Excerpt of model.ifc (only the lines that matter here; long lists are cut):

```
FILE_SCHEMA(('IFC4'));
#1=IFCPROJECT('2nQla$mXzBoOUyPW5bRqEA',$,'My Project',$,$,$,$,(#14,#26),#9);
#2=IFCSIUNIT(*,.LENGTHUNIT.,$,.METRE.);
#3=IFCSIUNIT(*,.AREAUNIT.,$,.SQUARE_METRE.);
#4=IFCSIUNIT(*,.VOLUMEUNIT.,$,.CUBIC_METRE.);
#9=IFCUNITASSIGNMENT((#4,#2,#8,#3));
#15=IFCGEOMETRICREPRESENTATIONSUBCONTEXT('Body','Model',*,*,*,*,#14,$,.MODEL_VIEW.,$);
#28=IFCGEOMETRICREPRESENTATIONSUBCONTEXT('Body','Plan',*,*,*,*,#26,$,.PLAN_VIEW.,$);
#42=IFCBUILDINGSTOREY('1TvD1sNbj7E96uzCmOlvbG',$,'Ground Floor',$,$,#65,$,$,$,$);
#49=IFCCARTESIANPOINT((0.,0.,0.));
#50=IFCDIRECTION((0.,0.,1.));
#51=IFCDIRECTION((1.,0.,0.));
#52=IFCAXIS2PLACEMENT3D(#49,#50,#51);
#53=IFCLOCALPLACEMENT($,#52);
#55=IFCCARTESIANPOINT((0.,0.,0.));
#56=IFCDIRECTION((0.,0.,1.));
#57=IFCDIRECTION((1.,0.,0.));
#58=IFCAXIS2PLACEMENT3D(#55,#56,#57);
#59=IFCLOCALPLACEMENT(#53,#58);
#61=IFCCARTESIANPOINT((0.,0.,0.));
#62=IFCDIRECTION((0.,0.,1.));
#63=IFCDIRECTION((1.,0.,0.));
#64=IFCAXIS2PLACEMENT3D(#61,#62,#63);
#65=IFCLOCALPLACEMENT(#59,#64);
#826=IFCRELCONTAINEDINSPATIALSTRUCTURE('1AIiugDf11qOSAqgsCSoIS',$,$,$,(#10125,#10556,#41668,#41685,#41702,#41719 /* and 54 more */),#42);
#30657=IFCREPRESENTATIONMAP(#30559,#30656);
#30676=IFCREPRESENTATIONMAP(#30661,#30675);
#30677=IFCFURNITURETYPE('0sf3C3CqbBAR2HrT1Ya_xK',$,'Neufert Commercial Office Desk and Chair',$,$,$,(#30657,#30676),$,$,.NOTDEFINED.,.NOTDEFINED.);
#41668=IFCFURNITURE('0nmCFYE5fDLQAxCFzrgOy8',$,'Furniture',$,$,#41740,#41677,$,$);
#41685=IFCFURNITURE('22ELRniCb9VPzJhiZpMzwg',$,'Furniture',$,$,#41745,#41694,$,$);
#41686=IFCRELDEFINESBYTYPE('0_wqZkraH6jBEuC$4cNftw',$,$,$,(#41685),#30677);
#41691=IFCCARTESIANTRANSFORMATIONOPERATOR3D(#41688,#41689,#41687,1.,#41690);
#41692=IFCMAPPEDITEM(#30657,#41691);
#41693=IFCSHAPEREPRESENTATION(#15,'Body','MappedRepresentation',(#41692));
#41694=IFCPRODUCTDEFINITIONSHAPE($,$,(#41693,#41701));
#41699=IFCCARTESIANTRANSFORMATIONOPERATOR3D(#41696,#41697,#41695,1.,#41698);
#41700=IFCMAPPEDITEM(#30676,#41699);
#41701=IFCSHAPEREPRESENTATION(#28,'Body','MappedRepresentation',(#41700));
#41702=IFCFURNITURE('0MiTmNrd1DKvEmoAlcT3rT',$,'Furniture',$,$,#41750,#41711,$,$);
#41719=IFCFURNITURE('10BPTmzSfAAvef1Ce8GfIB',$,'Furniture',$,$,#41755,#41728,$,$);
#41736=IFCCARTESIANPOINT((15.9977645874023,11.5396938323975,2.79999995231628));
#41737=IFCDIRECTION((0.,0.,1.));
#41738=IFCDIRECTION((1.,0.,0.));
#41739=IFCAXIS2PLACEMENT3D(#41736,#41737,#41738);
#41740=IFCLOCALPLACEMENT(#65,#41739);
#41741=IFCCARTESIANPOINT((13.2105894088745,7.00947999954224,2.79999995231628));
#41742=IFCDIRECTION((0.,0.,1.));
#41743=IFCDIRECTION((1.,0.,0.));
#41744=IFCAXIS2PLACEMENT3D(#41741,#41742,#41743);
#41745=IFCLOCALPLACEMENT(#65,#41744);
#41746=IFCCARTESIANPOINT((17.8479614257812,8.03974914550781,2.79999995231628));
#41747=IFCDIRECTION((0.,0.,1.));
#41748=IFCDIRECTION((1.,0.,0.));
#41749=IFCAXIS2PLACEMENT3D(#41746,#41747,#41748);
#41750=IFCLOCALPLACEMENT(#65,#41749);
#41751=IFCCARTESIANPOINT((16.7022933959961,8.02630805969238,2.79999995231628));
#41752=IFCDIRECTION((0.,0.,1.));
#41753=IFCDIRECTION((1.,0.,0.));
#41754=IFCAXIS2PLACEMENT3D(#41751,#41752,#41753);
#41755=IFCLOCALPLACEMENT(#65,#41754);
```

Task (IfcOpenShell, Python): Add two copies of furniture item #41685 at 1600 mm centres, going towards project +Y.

```python
import numpy as np
import ifcopenshell
import ifcopenshell.api.geometry
import ifcopenshell.api.root
import ifcopenshell.util.element
import ifcopenshell.util.placement
import ifcopenshell.util.unit

model = ifcopenshell.open("model.ifc")
unit_scale = ifcopenshell.util.unit.calculate_unit_scale(model)

source = model.by_id(41685)
base = ifcopenshell.util.placement.get_local_placement(source.ObjectPlacement)
step = np.array([0.0, 1.0, 0.0]) * 1.6 / unit_scale

for i in range(1, 3):
    copy = ifcopenshell.api.root.copy_class(model, product=source)
    copy.Representation = ifcopenshell.util.element.copy_deep(
        model, source.Representation, exclude=["IfcGeometricRepresentationContext", "IfcRepresentationMap"]
    )
    matrix = base.copy()
    matrix[:3, 3] += i * step
    print("added at", matrix[:3, 3].round(3) + 0.0)
    ifcopenshell.api.geometry.edit_object_placement(model, product=copy, matrix=matrix, is_si=False)

model.write("model_edited.ifc")
```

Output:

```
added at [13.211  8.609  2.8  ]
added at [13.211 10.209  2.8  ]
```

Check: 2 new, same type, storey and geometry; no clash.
